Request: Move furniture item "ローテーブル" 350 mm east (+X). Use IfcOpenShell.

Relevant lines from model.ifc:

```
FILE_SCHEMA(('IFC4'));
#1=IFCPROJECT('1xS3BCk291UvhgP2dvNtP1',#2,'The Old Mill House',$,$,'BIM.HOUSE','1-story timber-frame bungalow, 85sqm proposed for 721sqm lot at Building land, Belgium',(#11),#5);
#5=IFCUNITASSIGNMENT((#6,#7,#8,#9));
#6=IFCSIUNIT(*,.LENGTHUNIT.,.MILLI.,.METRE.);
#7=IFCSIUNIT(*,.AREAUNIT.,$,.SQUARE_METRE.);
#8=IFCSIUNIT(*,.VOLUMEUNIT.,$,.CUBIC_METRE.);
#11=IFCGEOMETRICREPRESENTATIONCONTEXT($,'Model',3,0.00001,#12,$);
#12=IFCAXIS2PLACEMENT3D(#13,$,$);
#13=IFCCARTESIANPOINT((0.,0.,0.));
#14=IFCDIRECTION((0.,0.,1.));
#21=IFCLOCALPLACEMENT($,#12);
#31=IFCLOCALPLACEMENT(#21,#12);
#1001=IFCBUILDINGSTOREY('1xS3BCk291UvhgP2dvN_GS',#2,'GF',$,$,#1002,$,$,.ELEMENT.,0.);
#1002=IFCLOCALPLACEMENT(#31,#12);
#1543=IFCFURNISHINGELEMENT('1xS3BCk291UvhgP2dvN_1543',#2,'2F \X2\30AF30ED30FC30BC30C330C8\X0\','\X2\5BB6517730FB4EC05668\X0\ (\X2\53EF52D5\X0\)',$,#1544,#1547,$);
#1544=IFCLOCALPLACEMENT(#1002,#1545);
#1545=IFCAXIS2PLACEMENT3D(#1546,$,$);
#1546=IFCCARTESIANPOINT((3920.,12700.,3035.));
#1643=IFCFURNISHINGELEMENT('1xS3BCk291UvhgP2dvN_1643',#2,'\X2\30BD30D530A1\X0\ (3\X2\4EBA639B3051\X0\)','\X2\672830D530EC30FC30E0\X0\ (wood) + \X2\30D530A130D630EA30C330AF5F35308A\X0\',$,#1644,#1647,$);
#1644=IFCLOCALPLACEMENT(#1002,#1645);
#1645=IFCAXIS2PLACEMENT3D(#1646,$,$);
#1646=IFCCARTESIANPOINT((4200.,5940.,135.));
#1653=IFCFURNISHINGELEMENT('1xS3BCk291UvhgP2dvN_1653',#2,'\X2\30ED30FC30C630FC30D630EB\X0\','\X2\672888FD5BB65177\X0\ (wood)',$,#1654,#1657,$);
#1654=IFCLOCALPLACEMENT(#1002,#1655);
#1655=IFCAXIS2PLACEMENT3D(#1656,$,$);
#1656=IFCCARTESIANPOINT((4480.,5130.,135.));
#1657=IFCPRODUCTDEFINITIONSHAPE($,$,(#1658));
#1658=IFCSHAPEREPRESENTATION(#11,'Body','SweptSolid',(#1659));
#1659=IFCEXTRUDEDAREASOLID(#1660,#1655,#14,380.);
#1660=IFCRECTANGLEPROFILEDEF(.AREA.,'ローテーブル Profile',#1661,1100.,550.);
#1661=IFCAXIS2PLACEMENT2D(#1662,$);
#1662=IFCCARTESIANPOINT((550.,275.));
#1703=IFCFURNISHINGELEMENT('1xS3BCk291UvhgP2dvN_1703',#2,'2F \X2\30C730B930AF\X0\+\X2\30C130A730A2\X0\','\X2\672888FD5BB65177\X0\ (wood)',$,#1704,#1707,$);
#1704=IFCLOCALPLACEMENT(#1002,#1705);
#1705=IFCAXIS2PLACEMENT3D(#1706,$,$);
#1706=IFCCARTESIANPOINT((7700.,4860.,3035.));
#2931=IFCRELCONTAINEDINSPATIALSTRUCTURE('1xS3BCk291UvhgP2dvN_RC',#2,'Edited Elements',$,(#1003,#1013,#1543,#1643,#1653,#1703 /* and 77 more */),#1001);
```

```python
import ifcopenshell
import ifcopenshell.api.geometry
import ifcopenshell.util.placement
import ifcopenshell.util.unit

model = ifcopenshell.open("model.ifc")
unit_scale = ifcopenshell.util.unit.calculate_unit_scale(model)

item = model.by_guid("1xS3BCk291UvhgP2dvN_1653")
matrix = ifcopenshell.util.placement.get_local_placement(item.ObjectPlacement)
matrix[0, 3] += 0.35 / unit_scale
ifcopenshell.api.geometry.edit_object_placement(model, product=item, matrix=matrix, is_si=False)

print(ifcopenshell.util.placement.get_local_placement(item.ObjectPlacement).round(3) + 0.0)

model.write("model_updated.ifc")
```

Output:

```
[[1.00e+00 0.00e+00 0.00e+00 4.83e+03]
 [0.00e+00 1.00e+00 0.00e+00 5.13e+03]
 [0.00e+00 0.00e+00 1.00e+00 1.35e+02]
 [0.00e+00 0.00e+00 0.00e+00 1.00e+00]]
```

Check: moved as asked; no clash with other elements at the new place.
